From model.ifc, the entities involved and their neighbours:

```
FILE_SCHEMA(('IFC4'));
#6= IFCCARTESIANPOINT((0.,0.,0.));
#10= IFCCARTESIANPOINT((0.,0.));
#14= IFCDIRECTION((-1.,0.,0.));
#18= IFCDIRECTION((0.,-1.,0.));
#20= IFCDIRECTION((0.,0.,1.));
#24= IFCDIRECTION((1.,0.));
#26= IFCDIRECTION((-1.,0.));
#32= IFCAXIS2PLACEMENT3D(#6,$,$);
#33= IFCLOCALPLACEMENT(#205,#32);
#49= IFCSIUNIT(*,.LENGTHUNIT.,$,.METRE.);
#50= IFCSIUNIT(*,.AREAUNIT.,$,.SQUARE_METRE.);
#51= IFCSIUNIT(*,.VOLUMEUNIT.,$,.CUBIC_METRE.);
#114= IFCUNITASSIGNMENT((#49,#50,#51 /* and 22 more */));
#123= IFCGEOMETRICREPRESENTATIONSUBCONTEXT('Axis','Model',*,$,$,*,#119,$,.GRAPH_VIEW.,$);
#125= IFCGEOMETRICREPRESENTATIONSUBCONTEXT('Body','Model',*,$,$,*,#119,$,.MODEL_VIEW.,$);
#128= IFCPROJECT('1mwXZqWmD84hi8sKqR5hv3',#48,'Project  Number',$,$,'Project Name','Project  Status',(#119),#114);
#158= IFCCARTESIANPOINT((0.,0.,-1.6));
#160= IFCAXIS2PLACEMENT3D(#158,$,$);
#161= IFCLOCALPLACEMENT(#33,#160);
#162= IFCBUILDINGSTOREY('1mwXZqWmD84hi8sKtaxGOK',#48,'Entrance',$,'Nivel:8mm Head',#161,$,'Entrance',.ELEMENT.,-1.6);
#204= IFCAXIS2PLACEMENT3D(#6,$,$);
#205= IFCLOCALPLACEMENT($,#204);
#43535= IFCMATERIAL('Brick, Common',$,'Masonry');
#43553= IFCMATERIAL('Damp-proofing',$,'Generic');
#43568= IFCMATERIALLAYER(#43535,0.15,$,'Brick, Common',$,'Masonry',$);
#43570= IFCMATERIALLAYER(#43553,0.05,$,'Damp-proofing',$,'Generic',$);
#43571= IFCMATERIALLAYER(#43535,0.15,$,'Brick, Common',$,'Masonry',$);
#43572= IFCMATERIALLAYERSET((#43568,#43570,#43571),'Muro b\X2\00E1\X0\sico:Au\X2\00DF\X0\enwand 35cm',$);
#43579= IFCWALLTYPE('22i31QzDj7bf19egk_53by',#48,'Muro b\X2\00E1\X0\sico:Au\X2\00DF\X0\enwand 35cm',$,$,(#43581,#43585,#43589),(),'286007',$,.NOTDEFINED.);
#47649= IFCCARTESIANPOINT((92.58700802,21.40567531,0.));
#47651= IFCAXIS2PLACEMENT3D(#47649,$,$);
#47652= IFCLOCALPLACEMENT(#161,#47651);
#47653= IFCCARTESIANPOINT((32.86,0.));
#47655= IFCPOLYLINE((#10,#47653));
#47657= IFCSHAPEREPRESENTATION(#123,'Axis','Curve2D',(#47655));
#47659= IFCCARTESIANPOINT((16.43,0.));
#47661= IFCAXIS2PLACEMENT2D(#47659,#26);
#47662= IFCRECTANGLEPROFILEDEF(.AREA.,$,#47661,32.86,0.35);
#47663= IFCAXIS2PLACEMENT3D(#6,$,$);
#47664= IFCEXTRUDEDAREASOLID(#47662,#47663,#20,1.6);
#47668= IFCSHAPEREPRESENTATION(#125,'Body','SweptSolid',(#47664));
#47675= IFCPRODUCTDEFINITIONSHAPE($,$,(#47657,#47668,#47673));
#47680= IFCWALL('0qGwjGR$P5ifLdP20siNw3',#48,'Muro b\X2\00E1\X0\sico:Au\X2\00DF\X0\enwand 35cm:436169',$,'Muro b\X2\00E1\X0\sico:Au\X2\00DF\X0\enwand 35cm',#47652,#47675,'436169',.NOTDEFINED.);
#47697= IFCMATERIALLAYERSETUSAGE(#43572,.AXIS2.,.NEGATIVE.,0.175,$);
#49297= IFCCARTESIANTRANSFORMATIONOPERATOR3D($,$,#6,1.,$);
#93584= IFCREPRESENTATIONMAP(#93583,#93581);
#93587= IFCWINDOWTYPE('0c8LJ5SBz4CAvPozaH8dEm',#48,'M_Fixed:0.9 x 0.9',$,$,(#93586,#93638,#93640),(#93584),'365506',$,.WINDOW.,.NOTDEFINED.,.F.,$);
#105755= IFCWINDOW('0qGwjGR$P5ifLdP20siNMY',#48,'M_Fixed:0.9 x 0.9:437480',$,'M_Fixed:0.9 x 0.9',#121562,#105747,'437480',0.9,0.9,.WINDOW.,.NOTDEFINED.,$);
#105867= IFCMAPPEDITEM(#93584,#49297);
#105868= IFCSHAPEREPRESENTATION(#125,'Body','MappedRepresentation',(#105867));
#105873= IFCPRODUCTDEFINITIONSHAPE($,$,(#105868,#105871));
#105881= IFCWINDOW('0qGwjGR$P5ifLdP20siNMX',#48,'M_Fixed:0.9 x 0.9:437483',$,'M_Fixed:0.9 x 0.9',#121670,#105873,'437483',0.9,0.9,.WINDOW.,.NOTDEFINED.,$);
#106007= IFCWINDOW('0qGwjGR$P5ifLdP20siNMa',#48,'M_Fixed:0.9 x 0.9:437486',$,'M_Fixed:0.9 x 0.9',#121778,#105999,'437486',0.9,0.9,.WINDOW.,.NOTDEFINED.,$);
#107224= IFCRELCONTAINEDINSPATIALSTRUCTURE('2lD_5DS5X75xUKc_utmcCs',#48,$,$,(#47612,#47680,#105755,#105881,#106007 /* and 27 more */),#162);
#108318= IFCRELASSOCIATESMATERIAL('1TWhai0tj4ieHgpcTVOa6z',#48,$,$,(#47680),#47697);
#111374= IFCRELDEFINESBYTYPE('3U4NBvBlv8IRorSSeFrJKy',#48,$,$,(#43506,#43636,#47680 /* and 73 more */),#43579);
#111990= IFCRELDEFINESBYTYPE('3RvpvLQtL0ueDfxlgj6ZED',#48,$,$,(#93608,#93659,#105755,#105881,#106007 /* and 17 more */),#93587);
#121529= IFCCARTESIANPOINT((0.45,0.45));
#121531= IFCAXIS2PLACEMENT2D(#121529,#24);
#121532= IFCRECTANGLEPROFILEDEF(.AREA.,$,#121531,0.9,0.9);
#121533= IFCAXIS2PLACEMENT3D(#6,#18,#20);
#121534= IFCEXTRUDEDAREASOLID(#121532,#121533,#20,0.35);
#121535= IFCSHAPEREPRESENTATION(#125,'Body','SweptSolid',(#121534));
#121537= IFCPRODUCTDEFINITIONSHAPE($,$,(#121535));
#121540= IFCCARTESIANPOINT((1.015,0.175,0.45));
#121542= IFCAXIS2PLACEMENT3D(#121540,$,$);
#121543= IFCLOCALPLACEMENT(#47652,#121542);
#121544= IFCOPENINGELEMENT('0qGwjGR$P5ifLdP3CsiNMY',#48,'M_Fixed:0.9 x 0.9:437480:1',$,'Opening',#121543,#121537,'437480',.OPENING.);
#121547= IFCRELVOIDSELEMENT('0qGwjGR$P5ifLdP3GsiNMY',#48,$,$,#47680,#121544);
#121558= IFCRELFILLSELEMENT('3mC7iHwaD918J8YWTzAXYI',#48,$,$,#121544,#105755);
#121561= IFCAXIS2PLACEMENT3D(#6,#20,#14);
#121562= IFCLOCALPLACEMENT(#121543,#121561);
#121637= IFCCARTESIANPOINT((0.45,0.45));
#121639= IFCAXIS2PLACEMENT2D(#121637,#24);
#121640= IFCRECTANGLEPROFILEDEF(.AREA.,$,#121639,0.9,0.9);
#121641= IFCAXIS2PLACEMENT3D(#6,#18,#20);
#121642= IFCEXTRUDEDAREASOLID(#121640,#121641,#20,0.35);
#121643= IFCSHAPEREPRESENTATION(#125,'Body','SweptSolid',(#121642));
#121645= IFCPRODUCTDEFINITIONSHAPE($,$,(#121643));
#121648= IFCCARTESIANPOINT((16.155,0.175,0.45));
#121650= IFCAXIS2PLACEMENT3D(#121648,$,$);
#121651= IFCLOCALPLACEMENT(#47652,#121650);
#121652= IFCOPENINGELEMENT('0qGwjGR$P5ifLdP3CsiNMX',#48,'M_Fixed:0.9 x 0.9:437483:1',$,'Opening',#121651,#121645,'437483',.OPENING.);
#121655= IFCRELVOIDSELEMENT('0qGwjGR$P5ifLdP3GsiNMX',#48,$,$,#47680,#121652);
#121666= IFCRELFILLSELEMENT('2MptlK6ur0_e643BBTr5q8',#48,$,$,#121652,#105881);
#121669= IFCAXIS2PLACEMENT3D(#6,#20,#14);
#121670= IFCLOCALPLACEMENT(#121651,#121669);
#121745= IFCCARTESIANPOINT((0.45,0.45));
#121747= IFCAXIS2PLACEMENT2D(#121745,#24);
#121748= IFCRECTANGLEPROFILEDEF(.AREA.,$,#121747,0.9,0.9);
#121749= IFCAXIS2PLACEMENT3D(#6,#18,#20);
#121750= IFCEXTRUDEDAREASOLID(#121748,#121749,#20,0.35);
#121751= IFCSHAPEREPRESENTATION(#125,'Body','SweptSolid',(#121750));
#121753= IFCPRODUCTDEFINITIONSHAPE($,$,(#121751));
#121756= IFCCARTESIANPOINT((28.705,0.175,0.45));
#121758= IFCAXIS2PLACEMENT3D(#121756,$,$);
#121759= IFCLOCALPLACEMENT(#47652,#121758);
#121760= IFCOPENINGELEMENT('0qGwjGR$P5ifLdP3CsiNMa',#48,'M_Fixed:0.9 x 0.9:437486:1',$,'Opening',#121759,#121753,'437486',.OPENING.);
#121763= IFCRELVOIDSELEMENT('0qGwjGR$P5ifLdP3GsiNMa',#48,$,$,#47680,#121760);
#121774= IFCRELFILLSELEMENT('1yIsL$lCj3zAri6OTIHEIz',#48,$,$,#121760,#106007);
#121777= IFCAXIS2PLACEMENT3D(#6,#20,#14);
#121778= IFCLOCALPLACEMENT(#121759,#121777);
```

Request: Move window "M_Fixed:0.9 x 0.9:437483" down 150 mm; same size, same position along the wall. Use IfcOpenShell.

```python
import numpy as np
import ifcopenshell
import ifcopenshell.api.geometry
import ifcopenshell.util.placement
import ifcopenshell.util.unit

model = ifcopenshell.open("model.ifc")
unit_scale = ifcopenshell.util.unit.calculate_unit_scale(model)

window = model.by_guid("0qGwjGR$P5ifLdP20siNMX")
opening = window.FillsVoids[0].RelatingOpeningElement
dz = -0.15 / unit_scale

shift = np.array([0.0, 0.0, dz])
# The window is placed relative to its opening, so it follows when the opening moves.
matrix = ifcopenshell.util.placement.get_local_placement(opening.ObjectPlacement)
matrix[:3, 3] += shift
ifcopenshell.api.geometry.edit_object_placement(
    model, product=opening, matrix=matrix, is_si=False, should_transform_children=True
)

print(f"moved by {dz * unit_scale:+.3f} m")

model.write("model-out.ifc")
```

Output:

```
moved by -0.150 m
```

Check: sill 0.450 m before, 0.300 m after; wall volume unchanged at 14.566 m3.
